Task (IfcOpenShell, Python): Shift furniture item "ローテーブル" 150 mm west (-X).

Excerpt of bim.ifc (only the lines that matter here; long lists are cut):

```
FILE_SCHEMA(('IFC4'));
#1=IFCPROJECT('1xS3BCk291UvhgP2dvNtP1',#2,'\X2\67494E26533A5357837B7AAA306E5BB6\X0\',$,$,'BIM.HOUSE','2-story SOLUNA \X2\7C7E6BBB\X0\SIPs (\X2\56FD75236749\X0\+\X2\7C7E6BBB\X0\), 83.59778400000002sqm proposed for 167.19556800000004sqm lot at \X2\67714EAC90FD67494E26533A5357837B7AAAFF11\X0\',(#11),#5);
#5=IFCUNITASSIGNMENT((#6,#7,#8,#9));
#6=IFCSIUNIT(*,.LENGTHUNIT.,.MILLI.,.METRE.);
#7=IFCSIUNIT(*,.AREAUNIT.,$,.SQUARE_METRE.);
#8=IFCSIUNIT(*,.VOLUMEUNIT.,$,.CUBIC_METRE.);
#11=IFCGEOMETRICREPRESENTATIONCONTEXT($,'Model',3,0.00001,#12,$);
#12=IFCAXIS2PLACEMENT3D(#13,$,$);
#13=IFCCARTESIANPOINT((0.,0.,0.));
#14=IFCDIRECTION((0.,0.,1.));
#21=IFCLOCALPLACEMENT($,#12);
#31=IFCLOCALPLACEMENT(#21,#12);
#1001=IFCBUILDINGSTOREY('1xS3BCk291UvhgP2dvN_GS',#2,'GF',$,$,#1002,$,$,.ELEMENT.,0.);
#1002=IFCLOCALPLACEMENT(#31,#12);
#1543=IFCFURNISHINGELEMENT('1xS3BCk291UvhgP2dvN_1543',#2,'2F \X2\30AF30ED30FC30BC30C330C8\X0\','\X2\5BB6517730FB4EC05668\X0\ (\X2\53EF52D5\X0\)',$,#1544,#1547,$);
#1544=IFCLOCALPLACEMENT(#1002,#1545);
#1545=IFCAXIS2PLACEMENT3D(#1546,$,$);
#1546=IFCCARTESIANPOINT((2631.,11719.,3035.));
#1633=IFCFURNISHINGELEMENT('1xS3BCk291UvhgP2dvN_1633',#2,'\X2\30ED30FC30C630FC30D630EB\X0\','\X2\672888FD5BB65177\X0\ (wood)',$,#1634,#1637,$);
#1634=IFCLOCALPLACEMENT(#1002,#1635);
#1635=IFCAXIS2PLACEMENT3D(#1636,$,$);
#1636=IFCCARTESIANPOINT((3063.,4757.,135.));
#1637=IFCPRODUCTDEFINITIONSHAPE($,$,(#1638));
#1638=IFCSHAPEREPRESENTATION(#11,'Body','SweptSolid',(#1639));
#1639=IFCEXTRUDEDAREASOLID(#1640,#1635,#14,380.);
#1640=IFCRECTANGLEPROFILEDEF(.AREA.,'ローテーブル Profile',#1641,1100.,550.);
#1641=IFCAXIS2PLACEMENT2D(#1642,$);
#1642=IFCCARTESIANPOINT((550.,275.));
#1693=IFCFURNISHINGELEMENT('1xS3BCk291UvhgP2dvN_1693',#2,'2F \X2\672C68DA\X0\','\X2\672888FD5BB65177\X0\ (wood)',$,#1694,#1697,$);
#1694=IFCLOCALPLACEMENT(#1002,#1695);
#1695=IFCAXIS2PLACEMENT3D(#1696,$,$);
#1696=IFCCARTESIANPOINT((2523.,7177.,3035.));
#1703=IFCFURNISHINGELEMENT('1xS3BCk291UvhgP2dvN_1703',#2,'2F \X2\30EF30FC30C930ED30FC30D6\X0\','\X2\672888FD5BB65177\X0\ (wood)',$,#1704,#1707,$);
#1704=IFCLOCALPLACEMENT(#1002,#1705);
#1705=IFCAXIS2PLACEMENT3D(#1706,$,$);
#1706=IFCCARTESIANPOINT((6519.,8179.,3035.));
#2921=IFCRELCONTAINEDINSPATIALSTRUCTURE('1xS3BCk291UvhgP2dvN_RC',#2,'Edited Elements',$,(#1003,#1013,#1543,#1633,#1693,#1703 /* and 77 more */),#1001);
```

```python
import ifcopenshell
import ifcopenshell.api.geometry
import ifcopenshell.util.placement
import ifcopenshell.util.unit

model = ifcopenshell.open("bim.ifc")
unit_scale = ifcopenshell.util.unit.calculate_unit_scale(model)

item = model.by_id(1633)
matrix = ifcopenshell.util.placement.get_local_placement(item.ObjectPlacement)
matrix[0, 3] -= 0.15 / unit_scale
ifcopenshell.api.geometry.edit_object_placement(model, product=item, matrix=matrix, is_si=False)

print(ifcopenshell.util.placement.get_local_placement(item.ObjectPlacement).round(3) + 0.0)

model.write("bim_edited.ifc")
```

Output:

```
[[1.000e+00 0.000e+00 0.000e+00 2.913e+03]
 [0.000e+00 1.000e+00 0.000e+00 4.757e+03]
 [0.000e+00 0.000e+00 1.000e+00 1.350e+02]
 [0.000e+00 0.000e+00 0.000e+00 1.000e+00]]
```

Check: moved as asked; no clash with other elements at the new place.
